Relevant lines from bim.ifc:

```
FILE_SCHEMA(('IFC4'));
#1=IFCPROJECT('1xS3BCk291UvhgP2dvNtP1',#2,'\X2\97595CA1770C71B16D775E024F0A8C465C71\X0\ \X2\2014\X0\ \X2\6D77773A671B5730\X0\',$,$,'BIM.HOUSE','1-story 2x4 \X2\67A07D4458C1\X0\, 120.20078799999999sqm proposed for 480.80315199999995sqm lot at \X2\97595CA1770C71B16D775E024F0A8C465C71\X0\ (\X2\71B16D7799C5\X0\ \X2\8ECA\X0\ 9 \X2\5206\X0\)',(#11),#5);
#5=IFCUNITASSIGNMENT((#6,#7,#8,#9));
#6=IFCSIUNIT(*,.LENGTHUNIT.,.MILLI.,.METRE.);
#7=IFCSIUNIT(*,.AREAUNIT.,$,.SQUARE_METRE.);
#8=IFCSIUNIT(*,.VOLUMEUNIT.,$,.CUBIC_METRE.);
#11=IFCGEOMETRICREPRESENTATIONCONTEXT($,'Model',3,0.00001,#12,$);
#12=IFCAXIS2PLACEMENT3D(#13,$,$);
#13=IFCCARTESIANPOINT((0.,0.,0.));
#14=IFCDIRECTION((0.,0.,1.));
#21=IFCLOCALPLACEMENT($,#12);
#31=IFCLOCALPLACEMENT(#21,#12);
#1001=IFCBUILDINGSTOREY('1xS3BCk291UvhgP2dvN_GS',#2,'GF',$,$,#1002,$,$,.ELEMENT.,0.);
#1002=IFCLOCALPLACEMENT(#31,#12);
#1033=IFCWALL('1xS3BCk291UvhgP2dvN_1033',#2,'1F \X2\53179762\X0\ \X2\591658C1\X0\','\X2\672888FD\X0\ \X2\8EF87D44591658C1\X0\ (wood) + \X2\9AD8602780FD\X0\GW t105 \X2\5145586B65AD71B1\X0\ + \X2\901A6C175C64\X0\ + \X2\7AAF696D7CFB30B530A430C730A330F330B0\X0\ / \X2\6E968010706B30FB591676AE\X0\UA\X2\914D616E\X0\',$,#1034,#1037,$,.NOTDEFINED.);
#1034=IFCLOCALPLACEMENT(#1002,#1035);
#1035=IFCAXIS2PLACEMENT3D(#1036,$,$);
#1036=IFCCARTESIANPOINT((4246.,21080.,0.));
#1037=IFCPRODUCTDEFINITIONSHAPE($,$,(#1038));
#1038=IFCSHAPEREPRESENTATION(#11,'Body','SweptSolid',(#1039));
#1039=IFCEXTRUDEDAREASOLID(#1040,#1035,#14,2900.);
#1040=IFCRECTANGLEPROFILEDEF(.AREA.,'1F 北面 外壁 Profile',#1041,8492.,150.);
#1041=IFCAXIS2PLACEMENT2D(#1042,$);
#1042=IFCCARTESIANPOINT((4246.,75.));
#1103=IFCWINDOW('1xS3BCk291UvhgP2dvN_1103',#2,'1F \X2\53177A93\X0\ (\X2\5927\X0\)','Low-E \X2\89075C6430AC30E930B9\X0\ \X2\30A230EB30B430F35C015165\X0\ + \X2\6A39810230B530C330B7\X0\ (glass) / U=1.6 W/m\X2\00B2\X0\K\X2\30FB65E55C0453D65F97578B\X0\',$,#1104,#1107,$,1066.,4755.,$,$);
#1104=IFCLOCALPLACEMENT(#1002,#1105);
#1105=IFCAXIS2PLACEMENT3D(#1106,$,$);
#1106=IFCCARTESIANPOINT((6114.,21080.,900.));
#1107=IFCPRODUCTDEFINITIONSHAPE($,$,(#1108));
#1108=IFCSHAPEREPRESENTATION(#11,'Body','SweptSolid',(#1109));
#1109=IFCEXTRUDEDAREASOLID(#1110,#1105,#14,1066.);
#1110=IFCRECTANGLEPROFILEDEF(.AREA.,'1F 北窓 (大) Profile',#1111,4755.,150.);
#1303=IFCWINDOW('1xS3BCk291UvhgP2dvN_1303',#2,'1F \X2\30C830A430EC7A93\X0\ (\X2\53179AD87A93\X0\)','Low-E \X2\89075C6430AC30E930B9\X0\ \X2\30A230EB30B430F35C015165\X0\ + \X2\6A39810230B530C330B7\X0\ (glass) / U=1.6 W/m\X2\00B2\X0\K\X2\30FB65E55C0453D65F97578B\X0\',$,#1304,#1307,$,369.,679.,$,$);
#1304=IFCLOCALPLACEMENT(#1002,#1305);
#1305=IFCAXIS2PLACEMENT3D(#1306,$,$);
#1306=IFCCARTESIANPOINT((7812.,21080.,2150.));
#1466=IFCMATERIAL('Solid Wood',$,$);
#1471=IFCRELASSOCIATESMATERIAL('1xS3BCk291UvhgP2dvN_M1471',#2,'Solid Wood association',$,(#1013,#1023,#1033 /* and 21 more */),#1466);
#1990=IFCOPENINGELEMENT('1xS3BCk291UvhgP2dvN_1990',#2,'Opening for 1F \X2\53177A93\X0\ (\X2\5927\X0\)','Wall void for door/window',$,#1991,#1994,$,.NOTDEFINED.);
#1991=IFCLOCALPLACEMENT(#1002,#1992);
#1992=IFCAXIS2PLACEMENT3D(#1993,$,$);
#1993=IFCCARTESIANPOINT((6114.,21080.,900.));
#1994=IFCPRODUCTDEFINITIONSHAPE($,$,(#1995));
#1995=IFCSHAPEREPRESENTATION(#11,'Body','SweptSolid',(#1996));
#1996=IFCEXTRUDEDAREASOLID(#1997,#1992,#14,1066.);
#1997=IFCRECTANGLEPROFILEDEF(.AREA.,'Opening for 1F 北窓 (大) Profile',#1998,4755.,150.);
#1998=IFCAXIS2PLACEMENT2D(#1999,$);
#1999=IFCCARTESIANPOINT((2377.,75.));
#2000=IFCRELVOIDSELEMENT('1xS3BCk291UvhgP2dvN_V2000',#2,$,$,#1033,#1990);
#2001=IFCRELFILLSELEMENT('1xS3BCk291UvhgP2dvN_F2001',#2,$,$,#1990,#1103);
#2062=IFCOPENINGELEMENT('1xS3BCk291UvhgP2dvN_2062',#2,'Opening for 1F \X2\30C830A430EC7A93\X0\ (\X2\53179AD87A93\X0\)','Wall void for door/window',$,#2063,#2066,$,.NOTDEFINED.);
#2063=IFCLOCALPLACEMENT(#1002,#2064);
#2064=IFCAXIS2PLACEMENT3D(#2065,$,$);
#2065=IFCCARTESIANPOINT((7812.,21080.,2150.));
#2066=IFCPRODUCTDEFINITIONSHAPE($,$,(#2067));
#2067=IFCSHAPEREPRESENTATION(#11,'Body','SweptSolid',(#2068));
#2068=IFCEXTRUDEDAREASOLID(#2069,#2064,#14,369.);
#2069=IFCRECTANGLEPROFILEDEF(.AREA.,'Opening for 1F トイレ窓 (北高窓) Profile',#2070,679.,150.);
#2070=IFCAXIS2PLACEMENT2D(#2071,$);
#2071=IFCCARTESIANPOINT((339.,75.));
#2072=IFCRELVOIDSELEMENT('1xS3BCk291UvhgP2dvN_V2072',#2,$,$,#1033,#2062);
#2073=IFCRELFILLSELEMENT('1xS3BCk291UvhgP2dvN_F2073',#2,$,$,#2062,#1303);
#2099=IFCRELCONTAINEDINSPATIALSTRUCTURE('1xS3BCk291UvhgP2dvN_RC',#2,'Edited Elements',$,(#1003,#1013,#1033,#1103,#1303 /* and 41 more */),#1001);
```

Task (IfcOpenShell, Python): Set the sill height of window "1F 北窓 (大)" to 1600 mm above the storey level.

```python
import numpy as np
import ifcopenshell
import ifcopenshell.api.geometry
import ifcopenshell.geom
import ifcopenshell.util.element
import ifcopenshell.util.placement
import ifcopenshell.util.shape
import ifcopenshell.util.unit

model = ifcopenshell.open("bim.ifc")
unit_scale = ifcopenshell.util.unit.calculate_unit_scale(model)

window = model.by_guid("1xS3BCk291UvhgP2dvN_1103")
opening = window.FillsVoids[0].RelatingOpeningElement
storey = ifcopenshell.util.element.get_container(window, ifc_class="IfcBuildingStorey")
level = ifcopenshell.util.placement.get_local_placement(storey.ObjectPlacement)[2, 3]

# The opening's origin need not be at the sill, so measure its lowest point.
shape = ifcopenshell.geom.create_shape(ifcopenshell.geom.settings(), opening)
bottom = ifcopenshell.util.shape.get_shape_bottom_elevation(shape, shape.geometry) / unit_scale
dz = level + 1.6 / unit_scale - bottom

shift = np.array([0.0, 0.0, dz])
# The window is not placed relative to its opening, so move both.
for product in (opening, window):
    matrix = ifcopenshell.util.placement.get_local_placement(product.ObjectPlacement)
    matrix[:3, 3] += shift
    ifcopenshell.api.geometry.edit_object_placement(model, product=product, matrix=matrix, is_si=False)

print(f"moved by {dz * unit_scale:+.3f} m")

model.write("bim_edited.ifc")
```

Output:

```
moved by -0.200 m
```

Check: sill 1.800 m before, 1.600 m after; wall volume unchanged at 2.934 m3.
